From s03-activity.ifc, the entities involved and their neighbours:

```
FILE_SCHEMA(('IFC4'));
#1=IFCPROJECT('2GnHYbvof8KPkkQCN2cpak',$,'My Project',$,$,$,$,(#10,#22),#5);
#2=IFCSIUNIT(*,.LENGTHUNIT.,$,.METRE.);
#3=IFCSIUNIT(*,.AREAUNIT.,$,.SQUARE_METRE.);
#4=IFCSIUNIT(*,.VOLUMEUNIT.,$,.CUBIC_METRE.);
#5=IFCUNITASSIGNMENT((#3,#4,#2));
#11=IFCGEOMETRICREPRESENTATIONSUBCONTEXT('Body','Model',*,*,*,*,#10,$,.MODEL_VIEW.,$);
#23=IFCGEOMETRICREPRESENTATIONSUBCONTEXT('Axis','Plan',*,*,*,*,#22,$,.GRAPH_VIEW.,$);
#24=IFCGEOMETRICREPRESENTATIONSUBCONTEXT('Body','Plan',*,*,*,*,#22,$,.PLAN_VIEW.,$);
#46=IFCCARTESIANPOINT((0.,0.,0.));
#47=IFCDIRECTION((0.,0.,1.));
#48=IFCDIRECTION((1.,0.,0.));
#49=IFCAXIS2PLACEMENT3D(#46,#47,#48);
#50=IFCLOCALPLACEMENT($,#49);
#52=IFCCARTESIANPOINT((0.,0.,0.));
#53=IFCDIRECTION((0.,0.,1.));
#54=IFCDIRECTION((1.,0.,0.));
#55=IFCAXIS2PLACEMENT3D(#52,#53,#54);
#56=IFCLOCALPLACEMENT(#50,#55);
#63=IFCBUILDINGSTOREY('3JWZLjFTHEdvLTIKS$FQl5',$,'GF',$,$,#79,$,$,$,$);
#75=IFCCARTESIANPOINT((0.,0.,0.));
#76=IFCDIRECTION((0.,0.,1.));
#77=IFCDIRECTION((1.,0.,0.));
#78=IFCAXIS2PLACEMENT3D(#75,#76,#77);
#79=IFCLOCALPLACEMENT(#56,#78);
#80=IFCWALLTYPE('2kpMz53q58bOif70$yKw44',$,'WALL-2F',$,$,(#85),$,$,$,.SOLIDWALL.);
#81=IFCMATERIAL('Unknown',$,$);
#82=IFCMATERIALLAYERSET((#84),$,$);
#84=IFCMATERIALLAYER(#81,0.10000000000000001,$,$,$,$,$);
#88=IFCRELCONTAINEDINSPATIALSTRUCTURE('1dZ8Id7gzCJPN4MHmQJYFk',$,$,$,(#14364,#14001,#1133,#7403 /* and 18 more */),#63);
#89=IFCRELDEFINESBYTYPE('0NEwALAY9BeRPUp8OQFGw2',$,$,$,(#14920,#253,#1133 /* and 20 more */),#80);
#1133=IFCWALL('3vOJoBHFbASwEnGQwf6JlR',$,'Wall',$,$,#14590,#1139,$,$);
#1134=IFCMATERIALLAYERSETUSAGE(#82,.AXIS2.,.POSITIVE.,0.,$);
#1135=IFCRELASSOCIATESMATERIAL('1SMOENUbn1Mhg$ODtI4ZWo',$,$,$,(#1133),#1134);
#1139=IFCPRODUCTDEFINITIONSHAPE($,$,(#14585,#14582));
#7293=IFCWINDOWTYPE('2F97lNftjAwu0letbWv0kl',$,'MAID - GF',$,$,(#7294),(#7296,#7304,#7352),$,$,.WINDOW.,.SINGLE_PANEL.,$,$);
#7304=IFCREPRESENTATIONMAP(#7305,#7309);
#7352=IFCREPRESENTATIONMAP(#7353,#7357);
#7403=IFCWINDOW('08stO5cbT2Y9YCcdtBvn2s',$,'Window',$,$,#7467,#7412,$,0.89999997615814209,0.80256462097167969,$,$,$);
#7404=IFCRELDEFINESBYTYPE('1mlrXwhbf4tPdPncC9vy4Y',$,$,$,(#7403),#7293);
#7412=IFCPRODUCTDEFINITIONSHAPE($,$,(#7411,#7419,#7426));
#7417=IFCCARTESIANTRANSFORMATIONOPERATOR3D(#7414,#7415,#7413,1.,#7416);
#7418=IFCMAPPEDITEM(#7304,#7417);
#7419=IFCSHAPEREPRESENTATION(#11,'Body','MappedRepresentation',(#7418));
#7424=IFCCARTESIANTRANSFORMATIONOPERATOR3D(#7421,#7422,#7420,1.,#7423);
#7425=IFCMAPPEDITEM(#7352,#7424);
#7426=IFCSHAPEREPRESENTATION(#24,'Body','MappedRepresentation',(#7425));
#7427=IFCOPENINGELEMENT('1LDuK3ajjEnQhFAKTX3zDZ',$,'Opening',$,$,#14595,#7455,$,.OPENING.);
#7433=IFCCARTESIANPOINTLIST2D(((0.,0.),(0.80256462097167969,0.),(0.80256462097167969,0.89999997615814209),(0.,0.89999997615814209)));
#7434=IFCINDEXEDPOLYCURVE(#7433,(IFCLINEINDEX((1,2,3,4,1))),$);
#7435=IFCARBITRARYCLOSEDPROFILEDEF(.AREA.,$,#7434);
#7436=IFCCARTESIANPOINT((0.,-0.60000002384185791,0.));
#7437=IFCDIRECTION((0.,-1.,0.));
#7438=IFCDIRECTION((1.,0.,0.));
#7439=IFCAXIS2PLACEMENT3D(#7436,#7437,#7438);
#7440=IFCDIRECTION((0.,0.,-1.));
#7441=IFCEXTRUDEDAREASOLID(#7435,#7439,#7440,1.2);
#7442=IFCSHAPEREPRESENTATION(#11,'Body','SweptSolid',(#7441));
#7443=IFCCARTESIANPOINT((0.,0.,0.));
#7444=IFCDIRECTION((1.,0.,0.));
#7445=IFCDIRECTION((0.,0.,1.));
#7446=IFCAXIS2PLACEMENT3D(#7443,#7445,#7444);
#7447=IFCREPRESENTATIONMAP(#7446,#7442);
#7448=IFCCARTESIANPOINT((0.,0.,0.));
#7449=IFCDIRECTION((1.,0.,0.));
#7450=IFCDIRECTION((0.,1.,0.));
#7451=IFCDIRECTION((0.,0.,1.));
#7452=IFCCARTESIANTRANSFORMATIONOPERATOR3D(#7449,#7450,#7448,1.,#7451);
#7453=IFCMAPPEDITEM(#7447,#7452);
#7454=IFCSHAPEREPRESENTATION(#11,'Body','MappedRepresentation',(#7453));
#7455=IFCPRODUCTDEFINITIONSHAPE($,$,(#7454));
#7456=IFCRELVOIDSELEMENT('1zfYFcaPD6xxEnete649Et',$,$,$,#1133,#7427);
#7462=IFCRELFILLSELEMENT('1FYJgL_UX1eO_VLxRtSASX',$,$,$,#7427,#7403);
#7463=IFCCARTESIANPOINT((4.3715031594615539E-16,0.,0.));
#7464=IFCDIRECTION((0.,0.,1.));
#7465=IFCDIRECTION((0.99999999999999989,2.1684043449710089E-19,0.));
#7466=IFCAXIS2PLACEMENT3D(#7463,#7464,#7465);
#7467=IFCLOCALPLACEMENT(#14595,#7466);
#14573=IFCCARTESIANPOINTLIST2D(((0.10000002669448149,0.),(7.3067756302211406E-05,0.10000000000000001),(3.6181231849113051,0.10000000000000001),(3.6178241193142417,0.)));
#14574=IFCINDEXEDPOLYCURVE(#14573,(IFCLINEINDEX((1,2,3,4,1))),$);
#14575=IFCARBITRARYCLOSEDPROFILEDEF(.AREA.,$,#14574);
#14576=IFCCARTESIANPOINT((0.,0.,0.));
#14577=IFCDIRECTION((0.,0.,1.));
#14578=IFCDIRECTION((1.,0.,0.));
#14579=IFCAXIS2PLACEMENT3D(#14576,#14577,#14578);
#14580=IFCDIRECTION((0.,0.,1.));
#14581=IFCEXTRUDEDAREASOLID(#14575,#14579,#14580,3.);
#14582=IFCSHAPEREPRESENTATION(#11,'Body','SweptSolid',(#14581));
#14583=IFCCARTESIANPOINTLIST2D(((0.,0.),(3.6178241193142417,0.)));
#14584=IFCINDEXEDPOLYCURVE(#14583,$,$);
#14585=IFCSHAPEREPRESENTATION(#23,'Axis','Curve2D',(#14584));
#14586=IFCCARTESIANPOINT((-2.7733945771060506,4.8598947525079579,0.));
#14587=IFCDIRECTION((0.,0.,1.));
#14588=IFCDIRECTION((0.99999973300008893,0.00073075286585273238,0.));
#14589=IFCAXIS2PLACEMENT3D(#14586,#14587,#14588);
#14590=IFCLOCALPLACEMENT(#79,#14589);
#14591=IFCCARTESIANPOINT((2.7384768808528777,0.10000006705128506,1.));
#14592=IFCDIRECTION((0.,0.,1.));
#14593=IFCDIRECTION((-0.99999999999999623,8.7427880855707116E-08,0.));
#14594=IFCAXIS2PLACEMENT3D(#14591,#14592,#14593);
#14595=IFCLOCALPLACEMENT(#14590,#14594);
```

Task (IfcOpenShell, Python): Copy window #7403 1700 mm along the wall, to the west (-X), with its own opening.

```python
import ifcopenshell
import ifcopenshell.api.feature
import ifcopenshell.api.geometry
import ifcopenshell.api.root
import ifcopenshell.geom
import ifcopenshell.util.element
import ifcopenshell.util.placement
import ifcopenshell.util.shape
import ifcopenshell.util.unit

model = ifcopenshell.open("s03-activity.ifc")
unit_scale = ifcopenshell.util.unit.calculate_unit_scale(model)
settings = ifcopenshell.geom.settings()


def volume(element):
    """Net volume in cubic metres, openings subtracted."""
    shape = ifcopenshell.geom.create_shape(settings, element)
    return ifcopenshell.util.shape.get_volume(shape.geometry)


window = model.by_guid("08stO5cbT2Y9YCcdtBvn2s")
opening = window.FillsVoids[0].RelatingOpeningElement
wall = opening.VoidsElements[0].RelatingBuildingElement
before = volume(wall)
shift = ifcopenshell.util.placement.get_local_placement(wall.ObjectPlacement)[:3, 0] * -1.7 / unit_scale

# copy_class copies the void relationship, type, container and properties, but no geometry.
new_opening = ifcopenshell.api.root.copy_class(model, product=opening)
new_opening.Representation = ifcopenshell.util.element.copy_deep(
    model, opening.Representation, exclude=["IfcGeometricRepresentationContext", "IfcRepresentationMap"]
)
new_window = ifcopenshell.api.root.copy_class(model, product=window)
new_window.Representation = ifcopenshell.util.element.copy_deep(
    model, window.Representation, exclude=["IfcGeometricRepresentationContext", "IfcRepresentationMap"]
)
ifcopenshell.api.feature.add_filling(model, opening=new_opening, element=new_window)

for old, new in ((opening, new_opening), (window, new_window)):
    matrix = ifcopenshell.util.placement.get_local_placement(old.ObjectPlacement)
    matrix[:3, 3] += shift
    ifcopenshell.api.geometry.edit_object_placement(model, product=new, matrix=matrix, is_si=False)

after = volume(wall)

print(f"wall volume {before:.3f} -> {after:.3f} m3")

model.write("s03-activity-out.ifc")
```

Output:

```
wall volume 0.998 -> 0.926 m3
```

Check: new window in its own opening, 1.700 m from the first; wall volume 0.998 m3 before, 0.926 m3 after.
